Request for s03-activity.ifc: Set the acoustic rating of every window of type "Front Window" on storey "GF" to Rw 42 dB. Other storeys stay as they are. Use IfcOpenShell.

First a look at what the model holds.

```python
import ifcopenshell
import ifcopenshell.util.element

model = ifcopenshell.open("s03-activity.ifc")
print(model.schema)
storey = next(s for s in model.by_type("IfcBuildingStorey") if s.Name == "GF")
windows = [e for e in ifcopenshell.util.element.get_decomposition(storey) if e.is_a("IfcWindow")]
seen = {}
for e in windows:
    element_type = ifcopenshell.util.element.get_type(e)
    key = (element_type.Name if element_type != e and element_type else None, ifcopenshell.util.element.get_pset(e, "Pset_WindowCommon", "AcousticRating"))
    seen[key] = seen.get(key, 0) + 1
for (name, value), count in sorted(seen.items(), key=str):
    print(count, "x", name, "|", value)
```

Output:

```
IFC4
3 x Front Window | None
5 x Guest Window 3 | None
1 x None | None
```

```python
import ifcopenshell
import ifcopenshell.api.pset
import ifcopenshell.util.element

model = ifcopenshell.open("s03-activity.ifc")

storey = next(s for s in model.by_type("IfcBuildingStorey") if s.Name == "GF")
windows = [e for e in ifcopenshell.util.element.get_decomposition(storey) if e.is_a("IfcWindow")]

count = 0
for e in windows:
    element_type = ifcopenshell.util.element.get_type(e)
    if element_type in (None, e) or element_type.Name != "Front Window":
        continue
    # add_pset returns the element's existing set when there is one.
    pset = ifcopenshell.api.pset.add_pset(model, product=e, name="Pset_WindowCommon")
    ifcopenshell.api.pset.edit_pset(model, pset=pset, properties={"AcousticRating": "Rw 42 dB"})
    count += 1

print(count, "windows updated")

model.write("s03-activity_v2.ifc")
```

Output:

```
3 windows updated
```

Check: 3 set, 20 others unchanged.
